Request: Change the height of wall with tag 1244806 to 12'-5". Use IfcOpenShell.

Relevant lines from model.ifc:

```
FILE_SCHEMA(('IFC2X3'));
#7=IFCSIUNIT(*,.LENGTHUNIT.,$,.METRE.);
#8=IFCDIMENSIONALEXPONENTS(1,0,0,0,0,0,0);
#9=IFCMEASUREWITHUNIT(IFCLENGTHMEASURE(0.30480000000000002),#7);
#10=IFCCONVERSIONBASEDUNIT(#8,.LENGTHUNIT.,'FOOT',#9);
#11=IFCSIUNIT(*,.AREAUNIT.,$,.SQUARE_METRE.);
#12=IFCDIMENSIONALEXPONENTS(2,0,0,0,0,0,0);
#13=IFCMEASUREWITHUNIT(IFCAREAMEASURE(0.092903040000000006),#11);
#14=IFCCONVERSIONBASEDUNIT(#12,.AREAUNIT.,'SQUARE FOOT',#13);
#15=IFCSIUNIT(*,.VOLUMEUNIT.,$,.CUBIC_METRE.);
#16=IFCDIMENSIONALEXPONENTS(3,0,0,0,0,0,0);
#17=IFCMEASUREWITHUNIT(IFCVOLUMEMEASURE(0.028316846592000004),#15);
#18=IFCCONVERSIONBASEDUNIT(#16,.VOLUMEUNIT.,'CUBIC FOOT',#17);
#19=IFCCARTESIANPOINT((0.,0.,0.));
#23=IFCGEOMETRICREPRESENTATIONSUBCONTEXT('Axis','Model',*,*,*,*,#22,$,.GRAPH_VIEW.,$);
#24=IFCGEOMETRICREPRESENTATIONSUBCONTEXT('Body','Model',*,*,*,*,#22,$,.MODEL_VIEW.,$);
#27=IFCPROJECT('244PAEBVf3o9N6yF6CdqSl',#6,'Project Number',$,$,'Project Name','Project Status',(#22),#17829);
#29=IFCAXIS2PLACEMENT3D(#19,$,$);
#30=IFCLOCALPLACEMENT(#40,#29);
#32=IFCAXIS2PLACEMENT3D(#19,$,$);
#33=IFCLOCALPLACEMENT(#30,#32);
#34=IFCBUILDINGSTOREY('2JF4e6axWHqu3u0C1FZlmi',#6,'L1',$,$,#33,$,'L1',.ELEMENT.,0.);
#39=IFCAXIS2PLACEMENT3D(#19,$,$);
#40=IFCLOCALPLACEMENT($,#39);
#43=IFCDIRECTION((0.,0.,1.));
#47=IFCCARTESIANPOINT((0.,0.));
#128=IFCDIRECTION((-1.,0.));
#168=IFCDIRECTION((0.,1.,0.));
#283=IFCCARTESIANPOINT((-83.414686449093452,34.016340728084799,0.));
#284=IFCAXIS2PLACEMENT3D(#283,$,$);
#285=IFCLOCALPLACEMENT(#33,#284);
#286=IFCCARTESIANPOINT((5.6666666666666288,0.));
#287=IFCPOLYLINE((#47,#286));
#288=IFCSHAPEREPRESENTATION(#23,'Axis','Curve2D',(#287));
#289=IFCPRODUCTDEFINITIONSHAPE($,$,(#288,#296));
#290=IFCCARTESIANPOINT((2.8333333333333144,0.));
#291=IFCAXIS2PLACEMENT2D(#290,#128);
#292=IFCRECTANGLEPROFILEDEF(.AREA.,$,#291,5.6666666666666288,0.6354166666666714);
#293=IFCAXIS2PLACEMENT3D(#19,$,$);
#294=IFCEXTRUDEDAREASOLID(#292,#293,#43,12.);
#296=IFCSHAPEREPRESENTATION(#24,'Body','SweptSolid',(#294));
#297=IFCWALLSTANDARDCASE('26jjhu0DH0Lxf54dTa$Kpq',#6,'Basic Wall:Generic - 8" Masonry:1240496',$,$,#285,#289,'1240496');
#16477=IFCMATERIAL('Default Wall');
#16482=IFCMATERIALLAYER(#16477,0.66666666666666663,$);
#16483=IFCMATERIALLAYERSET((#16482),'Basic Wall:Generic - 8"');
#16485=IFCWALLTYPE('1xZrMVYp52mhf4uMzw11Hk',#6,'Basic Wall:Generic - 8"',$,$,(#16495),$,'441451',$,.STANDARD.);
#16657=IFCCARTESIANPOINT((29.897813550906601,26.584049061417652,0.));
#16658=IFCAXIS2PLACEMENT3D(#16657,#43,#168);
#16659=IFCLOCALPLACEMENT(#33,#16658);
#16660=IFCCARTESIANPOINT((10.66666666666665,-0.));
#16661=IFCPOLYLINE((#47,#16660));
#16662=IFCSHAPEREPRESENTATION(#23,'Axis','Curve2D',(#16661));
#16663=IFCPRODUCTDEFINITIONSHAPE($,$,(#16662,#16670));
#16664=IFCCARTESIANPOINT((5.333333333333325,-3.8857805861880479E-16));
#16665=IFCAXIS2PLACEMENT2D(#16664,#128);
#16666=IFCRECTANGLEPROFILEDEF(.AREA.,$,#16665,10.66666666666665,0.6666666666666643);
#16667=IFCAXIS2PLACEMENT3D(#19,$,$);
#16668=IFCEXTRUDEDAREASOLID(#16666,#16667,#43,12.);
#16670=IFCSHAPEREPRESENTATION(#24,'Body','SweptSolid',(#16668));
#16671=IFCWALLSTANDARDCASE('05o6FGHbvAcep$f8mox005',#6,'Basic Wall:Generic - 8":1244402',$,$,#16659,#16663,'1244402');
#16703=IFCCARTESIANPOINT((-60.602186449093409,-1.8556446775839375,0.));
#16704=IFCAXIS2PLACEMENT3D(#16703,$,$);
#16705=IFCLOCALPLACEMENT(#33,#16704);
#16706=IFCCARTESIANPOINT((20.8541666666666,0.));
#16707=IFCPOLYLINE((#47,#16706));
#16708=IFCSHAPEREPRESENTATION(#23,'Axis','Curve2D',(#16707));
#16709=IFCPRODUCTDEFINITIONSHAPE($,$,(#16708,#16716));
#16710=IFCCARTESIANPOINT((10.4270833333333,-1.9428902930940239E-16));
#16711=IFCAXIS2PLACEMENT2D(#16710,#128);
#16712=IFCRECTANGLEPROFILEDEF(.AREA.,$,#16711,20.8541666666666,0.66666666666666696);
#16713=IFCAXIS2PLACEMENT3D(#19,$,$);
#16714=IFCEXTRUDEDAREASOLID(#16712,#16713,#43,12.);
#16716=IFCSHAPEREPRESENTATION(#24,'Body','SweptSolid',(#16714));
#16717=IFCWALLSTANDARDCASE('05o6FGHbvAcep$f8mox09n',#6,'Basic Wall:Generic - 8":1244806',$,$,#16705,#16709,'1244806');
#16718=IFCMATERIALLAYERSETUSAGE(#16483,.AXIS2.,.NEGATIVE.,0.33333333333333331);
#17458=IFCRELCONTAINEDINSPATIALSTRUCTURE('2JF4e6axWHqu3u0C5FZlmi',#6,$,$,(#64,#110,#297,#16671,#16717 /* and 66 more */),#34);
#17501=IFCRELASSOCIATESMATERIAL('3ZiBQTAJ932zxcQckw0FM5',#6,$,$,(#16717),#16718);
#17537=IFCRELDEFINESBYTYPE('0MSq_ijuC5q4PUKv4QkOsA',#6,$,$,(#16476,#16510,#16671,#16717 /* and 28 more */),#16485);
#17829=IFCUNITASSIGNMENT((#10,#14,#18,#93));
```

```python
import ifcopenshell
import ifcopenshell.geom
import ifcopenshell.util.representation
import ifcopenshell.util.shape
import ifcopenshell.util.unit

model = ifcopenshell.open("model.ifc")
unit_scale = ifcopenshell.util.unit.calculate_unit_scale(model)
settings = ifcopenshell.geom.settings()


def volume(element):
    """Net volume in cubic metres, openings subtracted."""
    shape = ifcopenshell.geom.create_shape(settings, element)
    return ifcopenshell.util.shape.get_volume(shape.geometry)


wall = model.by_guid("05o6FGHbvAcep$f8mox09n")
before = volume(wall)

body = ifcopenshell.util.representation.get_representation(wall, "Model", "Body")
solid = body.Items[0]
old_height = solid.Depth
solid.Depth = 149 * 0.0254 / unit_scale
after = volume(wall)

print(f"height {old_height:g} -> {solid.Depth:g}, volume {before:.3f} -> {after:.3f} m3")

model.write("model_v2.ifc")
```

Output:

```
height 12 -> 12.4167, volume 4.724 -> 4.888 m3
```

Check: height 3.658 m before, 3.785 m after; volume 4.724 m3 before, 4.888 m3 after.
